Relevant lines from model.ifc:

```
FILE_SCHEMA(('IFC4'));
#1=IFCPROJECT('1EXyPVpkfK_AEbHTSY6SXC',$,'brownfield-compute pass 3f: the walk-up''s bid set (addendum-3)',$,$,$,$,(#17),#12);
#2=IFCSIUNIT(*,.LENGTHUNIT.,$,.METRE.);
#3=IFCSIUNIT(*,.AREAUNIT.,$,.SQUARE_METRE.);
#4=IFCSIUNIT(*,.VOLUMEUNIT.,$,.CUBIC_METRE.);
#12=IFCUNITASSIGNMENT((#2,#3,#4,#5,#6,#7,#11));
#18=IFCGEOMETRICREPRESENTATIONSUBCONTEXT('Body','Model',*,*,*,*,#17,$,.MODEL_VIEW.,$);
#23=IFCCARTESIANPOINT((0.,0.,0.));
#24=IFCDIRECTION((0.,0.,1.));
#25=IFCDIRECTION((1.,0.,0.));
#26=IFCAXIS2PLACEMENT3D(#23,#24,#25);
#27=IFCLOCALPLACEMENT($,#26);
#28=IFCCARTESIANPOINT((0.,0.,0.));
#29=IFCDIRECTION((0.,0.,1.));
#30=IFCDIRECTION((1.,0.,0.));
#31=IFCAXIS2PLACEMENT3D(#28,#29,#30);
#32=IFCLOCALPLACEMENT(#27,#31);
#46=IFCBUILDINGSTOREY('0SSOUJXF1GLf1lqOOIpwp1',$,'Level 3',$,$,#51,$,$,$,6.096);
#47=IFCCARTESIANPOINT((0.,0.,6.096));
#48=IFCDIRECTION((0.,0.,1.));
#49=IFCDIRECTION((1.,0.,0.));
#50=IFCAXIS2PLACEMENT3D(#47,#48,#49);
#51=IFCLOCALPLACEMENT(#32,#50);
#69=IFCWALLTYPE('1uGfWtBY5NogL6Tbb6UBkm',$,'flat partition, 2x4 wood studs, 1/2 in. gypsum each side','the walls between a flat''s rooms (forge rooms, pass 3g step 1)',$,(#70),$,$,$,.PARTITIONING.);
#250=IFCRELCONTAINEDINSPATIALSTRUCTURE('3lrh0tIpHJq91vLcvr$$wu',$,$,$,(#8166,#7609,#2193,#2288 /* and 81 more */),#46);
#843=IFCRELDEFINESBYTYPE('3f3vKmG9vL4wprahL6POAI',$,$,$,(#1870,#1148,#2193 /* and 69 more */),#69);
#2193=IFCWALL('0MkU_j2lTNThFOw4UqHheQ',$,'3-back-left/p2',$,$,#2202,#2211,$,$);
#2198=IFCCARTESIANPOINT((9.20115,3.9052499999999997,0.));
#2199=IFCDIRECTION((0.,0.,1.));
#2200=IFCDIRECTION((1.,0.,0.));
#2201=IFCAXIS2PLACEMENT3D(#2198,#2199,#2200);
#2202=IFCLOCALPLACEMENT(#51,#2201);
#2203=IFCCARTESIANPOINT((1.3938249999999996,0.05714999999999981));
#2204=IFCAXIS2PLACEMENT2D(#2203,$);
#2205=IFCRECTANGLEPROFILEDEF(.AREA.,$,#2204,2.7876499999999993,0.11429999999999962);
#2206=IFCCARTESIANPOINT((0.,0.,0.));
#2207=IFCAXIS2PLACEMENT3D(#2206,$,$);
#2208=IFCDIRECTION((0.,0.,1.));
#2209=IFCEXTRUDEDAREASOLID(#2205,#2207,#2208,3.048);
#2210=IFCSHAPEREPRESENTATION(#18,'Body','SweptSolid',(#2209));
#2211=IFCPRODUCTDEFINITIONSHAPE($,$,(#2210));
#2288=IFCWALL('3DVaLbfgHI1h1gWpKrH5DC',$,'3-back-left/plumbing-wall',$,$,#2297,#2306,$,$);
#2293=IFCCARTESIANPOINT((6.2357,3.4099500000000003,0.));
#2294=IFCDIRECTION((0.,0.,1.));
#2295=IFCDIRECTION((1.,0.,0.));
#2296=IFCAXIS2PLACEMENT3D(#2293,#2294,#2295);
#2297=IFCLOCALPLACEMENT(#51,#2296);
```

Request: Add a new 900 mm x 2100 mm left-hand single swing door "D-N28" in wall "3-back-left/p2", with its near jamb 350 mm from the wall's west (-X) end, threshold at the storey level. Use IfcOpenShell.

```python
import numpy as np
import ifcopenshell
import ifcopenshell.api.feature
import ifcopenshell.api.geometry
import ifcopenshell.api.root
import ifcopenshell.api.spatial
import ifcopenshell.geom
import ifcopenshell.util.element
import ifcopenshell.util.placement
import ifcopenshell.util.representation
import ifcopenshell.util.shape
import ifcopenshell.util.unit

model = ifcopenshell.open("model.ifc")
unit_scale = ifcopenshell.util.unit.calculate_unit_scale(model)
settings = ifcopenshell.geom.settings()


def volume(element):
    """Net volume in cubic metres, openings subtracted."""
    shape = ifcopenshell.geom.create_shape(settings, element)
    return ifcopenshell.util.shape.get_volume(shape.geometry)


wall = model.by_guid("0MkU_j2lTNThFOw4UqHheQ")
storey = ifcopenshell.util.element.get_container(wall, ifc_class="IfcBuildingStorey")
context = ifcopenshell.util.representation.get_context(model, "Model", "Body", "MODEL_VIEW")
before = volume(wall)

width, height, from_end, sill = 0.9, 2.1, 0.35, 0.0  # metres

# The wall runs along its own X axis, and the end named is its -X end.
wall_shape = ifcopenshell.geom.create_shape(settings, wall)
x, y, z = ifcopenshell.util.shape.get_vertices(wall_shape.geometry).T
start = x.min() + from_end
face, thickness = float(y.min()), float(y.max() - y.min())
wall_matrix = ifcopenshell.util.placement.get_local_placement(wall.ObjectPlacement)
level = ifcopenshell.util.placement.get_local_placement(storey.ObjectPlacement)[2, 3]


def in_wall(x, y):
    """Placement at x, y metres in the wall's axes, at sill height."""
    matrix = wall_matrix.copy()
    matrix[:, 3] = wall_matrix @ np.array([x / unit_scale, y / unit_scale, 0.0, 1.0])
    matrix[2, 3] = level + sill / unit_scale
    return matrix


# Opening: a box that overshoots both wall faces by 50 mm.
opening = ifcopenshell.api.root.create_entity(model, ifc_class="IfcOpeningElement", predefined_type="OPENING")
box = ifcopenshell.api.geometry.add_wall_representation(
    model, context=context, length=width, height=height, thickness=thickness + 0.1
)
ifcopenshell.api.geometry.assign_representation(model, product=opening, representation=box)
ifcopenshell.api.geometry.edit_object_placement(model, product=opening, matrix=in_wall(start, face - 0.05), is_si=False)
ifcopenshell.api.feature.add_feature(model, feature=opening, element=wall)

door = ifcopenshell.api.root.create_entity(model, ifc_class="IfcDoor", name="D-N28", predefined_type="DOOR")
door.OverallWidth, door.OverallHeight = width / unit_scale, height / unit_scale
door.OperationType = "SINGLE_SWING_LEFT"
body = ifcopenshell.api.geometry.add_door_representation(
    model,
    context=context,
    overall_width=door.OverallWidth,
    overall_height=door.OverallHeight,
    operation_type="SINGLE_SWING_LEFT",
    lining_properties={"LiningDepth": thickness / unit_scale, "ThresholdDepth": thickness / unit_scale},
)
ifcopenshell.api.geometry.assign_representation(model, product=door, representation=body)
ifcopenshell.api.spatial.assign_container(model, products=[door], relating_structure=storey)
ifcopenshell.api.feature.add_filling(model, opening=opening, element=door)

# The lining spans the wall, so the door starts at the wall face.
ifcopenshell.api.geometry.edit_object_placement(model, product=door, matrix=in_wall(start, face), is_si=False)

after = volume(wall)

print(f"wall volume {before:.3f} -> {after:.3f} m3")

model.write("model_updated.ifc")
```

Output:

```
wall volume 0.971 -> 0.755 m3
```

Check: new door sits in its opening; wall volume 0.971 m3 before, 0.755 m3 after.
